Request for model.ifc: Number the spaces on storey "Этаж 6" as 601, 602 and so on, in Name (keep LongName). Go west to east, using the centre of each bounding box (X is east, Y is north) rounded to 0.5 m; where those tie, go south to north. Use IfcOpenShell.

First a look at what the model holds.

```python
import ifcopenshell
import ifcopenshell.util.element
import ifcopenshell.util.placement

model = ifcopenshell.open("model.ifc")
print(model.schema)
storey = next(s for s in model.by_type("IfcBuildingStorey") if s.Name == "Этаж 6")
spaces = [e for e in ifcopenshell.util.element.get_decomposition(storey) if e.is_a("IfcSpace")]
for e in sorted(spaces, key=lambda e: e.id()):
    origin = ifcopenshell.util.placement.get_local_placement(e.ObjectPlacement)[:3, 3]
    print(e.id(), e.Name, e.LongName, origin.round(2) + 0.0, sep=" | ")
```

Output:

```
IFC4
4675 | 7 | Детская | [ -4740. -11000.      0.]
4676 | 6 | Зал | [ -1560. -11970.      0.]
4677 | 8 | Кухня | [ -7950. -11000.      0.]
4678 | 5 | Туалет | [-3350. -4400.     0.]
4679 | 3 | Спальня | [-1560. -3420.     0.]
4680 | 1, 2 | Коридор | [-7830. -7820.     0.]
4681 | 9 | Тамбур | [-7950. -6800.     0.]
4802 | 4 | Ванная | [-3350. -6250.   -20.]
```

```python
import ifcopenshell
import ifcopenshell.geom
import ifcopenshell.util.element
import ifcopenshell.util.shape

model = ifcopenshell.open("model.ifc")
settings = ifcopenshell.geom.settings()
settings.set("use-world-coords", True)


def centre(element):
    shape = ifcopenshell.geom.create_shape(settings, element)
    return ifcopenshell.util.shape.get_bbox_centroid(shape.geometry)


storey = next(s for s in model.by_type("IfcBuildingStorey") if s.Name == "Этаж 6")
spaces = [e for e in ifcopenshell.util.element.get_decomposition(storey) if e.is_a("IfcSpace")]

# Insertion points can sit at a corner or the storey origin, so sort by the geometry (in metres).
centres = {e: centre(e) for e in spaces}
spaces.sort(key=lambda e: (round(centres[e][0] / 0.5), centres[e][1]))

for i, e in enumerate(spaces, start=1):
    number = f"6{i:02d}"
    e.Name = number
    print(e.id(), number)

model.write("model_rev.ifc")
```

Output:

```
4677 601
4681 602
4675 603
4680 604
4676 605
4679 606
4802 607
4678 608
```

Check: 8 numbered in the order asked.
